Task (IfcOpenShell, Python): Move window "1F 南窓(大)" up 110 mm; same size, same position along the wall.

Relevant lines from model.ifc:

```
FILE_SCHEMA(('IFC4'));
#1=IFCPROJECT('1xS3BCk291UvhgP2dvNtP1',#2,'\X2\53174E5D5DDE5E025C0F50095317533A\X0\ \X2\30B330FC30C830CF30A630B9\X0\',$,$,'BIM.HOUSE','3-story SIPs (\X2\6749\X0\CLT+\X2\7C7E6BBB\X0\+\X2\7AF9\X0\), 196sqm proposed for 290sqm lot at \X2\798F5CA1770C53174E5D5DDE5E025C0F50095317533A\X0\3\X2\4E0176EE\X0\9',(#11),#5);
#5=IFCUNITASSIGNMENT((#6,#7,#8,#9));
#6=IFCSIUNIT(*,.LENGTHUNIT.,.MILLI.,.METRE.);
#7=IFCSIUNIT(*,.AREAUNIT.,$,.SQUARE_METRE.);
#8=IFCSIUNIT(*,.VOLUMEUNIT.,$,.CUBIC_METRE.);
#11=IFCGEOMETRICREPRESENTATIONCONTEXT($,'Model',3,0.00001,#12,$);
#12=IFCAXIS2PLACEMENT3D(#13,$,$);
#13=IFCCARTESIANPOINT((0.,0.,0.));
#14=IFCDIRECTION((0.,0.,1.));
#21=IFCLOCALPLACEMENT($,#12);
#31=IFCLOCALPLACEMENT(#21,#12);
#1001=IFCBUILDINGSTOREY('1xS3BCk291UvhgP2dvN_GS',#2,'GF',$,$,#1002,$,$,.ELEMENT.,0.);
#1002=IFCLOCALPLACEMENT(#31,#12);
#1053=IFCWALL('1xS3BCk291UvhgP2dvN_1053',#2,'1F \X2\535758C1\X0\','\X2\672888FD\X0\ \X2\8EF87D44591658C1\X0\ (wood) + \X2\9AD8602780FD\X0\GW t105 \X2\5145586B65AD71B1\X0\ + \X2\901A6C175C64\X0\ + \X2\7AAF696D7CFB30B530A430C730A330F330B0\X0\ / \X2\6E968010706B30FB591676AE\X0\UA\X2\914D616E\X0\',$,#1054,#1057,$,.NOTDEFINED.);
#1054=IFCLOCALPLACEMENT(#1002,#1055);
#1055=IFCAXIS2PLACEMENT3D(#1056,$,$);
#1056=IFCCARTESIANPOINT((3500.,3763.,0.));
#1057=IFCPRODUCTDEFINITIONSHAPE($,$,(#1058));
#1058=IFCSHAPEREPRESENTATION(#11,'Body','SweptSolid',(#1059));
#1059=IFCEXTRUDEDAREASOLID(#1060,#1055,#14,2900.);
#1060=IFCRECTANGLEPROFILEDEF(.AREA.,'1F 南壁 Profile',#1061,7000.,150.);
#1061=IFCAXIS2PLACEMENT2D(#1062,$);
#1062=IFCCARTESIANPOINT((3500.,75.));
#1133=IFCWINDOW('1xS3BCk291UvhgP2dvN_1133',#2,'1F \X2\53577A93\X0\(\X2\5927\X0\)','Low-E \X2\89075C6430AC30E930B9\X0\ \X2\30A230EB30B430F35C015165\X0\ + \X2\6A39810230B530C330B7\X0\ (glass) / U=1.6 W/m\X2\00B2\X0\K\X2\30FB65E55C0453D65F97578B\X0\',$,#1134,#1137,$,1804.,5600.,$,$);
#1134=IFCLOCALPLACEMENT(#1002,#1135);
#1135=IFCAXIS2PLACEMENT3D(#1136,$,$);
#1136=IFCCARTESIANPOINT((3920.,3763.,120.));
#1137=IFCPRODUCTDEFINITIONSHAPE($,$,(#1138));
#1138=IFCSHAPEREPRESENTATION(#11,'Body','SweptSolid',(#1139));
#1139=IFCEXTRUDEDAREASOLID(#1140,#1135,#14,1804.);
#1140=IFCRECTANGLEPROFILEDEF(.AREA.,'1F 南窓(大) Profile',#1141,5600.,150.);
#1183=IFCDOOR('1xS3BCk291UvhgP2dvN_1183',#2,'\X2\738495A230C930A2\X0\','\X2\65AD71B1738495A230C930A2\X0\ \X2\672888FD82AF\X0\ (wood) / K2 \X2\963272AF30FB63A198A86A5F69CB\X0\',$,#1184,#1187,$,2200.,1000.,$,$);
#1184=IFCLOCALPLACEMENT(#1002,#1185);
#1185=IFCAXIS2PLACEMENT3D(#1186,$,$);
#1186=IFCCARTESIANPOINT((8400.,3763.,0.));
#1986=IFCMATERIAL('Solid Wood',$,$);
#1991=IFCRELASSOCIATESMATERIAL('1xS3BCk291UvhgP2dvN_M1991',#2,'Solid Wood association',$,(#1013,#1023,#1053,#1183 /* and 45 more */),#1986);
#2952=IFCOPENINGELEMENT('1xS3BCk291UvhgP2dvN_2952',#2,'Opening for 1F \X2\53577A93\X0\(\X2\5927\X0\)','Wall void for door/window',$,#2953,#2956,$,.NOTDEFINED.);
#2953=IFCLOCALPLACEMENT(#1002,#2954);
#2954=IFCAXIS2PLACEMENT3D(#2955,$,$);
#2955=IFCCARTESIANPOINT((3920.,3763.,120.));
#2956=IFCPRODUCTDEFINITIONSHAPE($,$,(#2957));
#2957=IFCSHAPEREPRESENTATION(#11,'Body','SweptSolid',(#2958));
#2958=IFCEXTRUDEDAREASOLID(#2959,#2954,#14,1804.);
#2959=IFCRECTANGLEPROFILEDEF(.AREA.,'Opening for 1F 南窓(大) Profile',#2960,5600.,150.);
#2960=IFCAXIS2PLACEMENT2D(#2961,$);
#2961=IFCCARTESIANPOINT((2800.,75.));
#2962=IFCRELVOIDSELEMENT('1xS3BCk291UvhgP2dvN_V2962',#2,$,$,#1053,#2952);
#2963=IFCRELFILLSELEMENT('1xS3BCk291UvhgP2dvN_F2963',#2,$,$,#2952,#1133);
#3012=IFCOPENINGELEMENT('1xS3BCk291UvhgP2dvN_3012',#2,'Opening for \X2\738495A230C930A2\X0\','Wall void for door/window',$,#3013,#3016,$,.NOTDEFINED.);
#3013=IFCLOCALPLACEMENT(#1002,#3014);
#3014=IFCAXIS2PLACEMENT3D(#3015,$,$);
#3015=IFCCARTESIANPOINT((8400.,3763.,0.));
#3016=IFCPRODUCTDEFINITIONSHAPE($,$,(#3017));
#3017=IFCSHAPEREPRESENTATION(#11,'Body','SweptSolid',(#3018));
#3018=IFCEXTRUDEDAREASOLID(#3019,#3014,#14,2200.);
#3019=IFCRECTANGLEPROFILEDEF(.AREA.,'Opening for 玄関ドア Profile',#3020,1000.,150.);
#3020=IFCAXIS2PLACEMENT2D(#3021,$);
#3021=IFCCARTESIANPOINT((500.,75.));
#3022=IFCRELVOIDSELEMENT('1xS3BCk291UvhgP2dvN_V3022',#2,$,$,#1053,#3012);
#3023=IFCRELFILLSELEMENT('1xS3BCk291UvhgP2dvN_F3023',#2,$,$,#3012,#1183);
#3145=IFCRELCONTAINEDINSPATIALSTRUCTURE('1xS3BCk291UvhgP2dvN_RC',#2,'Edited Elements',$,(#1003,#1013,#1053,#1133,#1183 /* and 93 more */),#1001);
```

```python
import numpy as np
import ifcopenshell
import ifcopenshell.api.geometry
import ifcopenshell.util.placement
import ifcopenshell.util.unit

model = ifcopenshell.open("model.ifc")
unit_scale = ifcopenshell.util.unit.calculate_unit_scale(model)

window = model.by_guid("1xS3BCk291UvhgP2dvN_1133")
opening = window.FillsVoids[0].RelatingOpeningElement
dz = 110.0

shift = np.array([0.0, 0.0, dz])
# The window is not placed relative to its opening, so move both.
for product in (opening, window):
    matrix = ifcopenshell.util.placement.get_local_placement(product.ObjectPlacement)
    matrix[:3, 3] += shift
    ifcopenshell.api.geometry.edit_object_placement(model, product=product, matrix=matrix, is_si=False)

print(f"moved by {dz * unit_scale:+.3f} m")

model.write("model-out.ifc")
```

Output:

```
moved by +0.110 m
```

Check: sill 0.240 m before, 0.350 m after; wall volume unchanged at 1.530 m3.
